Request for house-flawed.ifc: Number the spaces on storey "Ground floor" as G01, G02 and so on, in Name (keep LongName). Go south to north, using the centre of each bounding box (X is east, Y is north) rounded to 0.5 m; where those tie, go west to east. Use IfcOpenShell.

First a look at what the model holds.

```python
import ifcopenshell
import ifcopenshell.util.element
import ifcopenshell.util.placement

model = ifcopenshell.open("house-flawed.ifc")
print(model.schema)
storey = next(s for s in model.by_type("IfcBuildingStorey") if s.Name == "Ground floor")
spaces = [e for e in ifcopenshell.util.element.get_decomposition(storey) if e.is_a("IfcSpace")]
for e in sorted(spaces, key=lambda e: e.id()):
    origin = ifcopenshell.util.placement.get_local_placement(e.ObjectPlacement)[:3, 3]
    print(e.id(), e.Name, e.LongName, origin.round(2) + 0.0, sep=" | ")
```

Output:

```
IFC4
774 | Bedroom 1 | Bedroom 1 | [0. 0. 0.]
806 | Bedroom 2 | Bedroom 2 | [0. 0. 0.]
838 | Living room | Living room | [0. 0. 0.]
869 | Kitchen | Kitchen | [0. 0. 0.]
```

```python
import ifcopenshell
import ifcopenshell.geom
import ifcopenshell.util.element
import ifcopenshell.util.shape

model = ifcopenshell.open("house-flawed.ifc")
settings = ifcopenshell.geom.settings()
settings.set("use-world-coords", True)


def centre(element):
    shape = ifcopenshell.geom.create_shape(settings, element)
    return ifcopenshell.util.shape.get_bbox_centroid(shape.geometry)


storey = next(s for s in model.by_type("IfcBuildingStorey") if s.Name == "Ground floor")
spaces = [e for e in ifcopenshell.util.element.get_decomposition(storey) if e.is_a("IfcSpace")]

# Insertion points can sit at a corner or the storey origin, so sort by the geometry (in metres).
centres = {e: centre(e) for e in spaces}
spaces.sort(key=lambda e: (round(centres[e][1] / 0.5), centres[e][0]))

for i, e in enumerate(spaces, start=1):
    number = f"G{i:02d}"
    e.Name = number
    print(e.id(), number)

model.write("house-flawed_updated.ifc")
```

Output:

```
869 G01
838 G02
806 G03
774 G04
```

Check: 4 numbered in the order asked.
